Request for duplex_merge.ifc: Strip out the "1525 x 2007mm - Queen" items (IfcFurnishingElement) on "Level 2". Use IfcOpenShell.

First a look at what the model holds.

```python
import ifcopenshell
import ifcopenshell.util.element

model = ifcopenshell.open("duplex_merge.ifc")
print(model.schema)
storey = next(s for s in model.by_type("IfcBuildingStorey") if s.Name == "Level 2")
furniture = [e for e in ifcopenshell.util.element.get_decomposition(storey) if e.is_a("IfcFurnishingElement")]
seen = {}
for e in furniture:
    element_type = ifcopenshell.util.element.get_type(e)
    name = element_type.Name if element_type not in (None, e) else None
    seen[name] = seen.get(name, 0) + 1
for name, count in sorted(seen.items(), key=str):
    print(count, "x", name)
```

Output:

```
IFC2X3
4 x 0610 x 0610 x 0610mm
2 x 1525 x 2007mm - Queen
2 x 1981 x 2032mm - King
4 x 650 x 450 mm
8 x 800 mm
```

```python
import ifcopenshell
import ifcopenshell.api.root
import ifcopenshell.util.element

model = ifcopenshell.open("duplex_merge.ifc")

storey = next(s for s in model.by_type("IfcBuildingStorey") if s.Name == "Level 2")
furniture = [e for e in ifcopenshell.util.element.get_decomposition(storey) if e.is_a("IfcFurnishingElement")]
targets = [e for e in furniture if (t := ifcopenshell.util.element.get_type(e)) not in (None, e) and t.Name == "1525 x 2007mm - Queen"]

for e in targets:
    ifcopenshell.api.root.remove_product(model, product=e)
print(len(targets), "removed")

model.write("duplex_merge_updated.ifc")
```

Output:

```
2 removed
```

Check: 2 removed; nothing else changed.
